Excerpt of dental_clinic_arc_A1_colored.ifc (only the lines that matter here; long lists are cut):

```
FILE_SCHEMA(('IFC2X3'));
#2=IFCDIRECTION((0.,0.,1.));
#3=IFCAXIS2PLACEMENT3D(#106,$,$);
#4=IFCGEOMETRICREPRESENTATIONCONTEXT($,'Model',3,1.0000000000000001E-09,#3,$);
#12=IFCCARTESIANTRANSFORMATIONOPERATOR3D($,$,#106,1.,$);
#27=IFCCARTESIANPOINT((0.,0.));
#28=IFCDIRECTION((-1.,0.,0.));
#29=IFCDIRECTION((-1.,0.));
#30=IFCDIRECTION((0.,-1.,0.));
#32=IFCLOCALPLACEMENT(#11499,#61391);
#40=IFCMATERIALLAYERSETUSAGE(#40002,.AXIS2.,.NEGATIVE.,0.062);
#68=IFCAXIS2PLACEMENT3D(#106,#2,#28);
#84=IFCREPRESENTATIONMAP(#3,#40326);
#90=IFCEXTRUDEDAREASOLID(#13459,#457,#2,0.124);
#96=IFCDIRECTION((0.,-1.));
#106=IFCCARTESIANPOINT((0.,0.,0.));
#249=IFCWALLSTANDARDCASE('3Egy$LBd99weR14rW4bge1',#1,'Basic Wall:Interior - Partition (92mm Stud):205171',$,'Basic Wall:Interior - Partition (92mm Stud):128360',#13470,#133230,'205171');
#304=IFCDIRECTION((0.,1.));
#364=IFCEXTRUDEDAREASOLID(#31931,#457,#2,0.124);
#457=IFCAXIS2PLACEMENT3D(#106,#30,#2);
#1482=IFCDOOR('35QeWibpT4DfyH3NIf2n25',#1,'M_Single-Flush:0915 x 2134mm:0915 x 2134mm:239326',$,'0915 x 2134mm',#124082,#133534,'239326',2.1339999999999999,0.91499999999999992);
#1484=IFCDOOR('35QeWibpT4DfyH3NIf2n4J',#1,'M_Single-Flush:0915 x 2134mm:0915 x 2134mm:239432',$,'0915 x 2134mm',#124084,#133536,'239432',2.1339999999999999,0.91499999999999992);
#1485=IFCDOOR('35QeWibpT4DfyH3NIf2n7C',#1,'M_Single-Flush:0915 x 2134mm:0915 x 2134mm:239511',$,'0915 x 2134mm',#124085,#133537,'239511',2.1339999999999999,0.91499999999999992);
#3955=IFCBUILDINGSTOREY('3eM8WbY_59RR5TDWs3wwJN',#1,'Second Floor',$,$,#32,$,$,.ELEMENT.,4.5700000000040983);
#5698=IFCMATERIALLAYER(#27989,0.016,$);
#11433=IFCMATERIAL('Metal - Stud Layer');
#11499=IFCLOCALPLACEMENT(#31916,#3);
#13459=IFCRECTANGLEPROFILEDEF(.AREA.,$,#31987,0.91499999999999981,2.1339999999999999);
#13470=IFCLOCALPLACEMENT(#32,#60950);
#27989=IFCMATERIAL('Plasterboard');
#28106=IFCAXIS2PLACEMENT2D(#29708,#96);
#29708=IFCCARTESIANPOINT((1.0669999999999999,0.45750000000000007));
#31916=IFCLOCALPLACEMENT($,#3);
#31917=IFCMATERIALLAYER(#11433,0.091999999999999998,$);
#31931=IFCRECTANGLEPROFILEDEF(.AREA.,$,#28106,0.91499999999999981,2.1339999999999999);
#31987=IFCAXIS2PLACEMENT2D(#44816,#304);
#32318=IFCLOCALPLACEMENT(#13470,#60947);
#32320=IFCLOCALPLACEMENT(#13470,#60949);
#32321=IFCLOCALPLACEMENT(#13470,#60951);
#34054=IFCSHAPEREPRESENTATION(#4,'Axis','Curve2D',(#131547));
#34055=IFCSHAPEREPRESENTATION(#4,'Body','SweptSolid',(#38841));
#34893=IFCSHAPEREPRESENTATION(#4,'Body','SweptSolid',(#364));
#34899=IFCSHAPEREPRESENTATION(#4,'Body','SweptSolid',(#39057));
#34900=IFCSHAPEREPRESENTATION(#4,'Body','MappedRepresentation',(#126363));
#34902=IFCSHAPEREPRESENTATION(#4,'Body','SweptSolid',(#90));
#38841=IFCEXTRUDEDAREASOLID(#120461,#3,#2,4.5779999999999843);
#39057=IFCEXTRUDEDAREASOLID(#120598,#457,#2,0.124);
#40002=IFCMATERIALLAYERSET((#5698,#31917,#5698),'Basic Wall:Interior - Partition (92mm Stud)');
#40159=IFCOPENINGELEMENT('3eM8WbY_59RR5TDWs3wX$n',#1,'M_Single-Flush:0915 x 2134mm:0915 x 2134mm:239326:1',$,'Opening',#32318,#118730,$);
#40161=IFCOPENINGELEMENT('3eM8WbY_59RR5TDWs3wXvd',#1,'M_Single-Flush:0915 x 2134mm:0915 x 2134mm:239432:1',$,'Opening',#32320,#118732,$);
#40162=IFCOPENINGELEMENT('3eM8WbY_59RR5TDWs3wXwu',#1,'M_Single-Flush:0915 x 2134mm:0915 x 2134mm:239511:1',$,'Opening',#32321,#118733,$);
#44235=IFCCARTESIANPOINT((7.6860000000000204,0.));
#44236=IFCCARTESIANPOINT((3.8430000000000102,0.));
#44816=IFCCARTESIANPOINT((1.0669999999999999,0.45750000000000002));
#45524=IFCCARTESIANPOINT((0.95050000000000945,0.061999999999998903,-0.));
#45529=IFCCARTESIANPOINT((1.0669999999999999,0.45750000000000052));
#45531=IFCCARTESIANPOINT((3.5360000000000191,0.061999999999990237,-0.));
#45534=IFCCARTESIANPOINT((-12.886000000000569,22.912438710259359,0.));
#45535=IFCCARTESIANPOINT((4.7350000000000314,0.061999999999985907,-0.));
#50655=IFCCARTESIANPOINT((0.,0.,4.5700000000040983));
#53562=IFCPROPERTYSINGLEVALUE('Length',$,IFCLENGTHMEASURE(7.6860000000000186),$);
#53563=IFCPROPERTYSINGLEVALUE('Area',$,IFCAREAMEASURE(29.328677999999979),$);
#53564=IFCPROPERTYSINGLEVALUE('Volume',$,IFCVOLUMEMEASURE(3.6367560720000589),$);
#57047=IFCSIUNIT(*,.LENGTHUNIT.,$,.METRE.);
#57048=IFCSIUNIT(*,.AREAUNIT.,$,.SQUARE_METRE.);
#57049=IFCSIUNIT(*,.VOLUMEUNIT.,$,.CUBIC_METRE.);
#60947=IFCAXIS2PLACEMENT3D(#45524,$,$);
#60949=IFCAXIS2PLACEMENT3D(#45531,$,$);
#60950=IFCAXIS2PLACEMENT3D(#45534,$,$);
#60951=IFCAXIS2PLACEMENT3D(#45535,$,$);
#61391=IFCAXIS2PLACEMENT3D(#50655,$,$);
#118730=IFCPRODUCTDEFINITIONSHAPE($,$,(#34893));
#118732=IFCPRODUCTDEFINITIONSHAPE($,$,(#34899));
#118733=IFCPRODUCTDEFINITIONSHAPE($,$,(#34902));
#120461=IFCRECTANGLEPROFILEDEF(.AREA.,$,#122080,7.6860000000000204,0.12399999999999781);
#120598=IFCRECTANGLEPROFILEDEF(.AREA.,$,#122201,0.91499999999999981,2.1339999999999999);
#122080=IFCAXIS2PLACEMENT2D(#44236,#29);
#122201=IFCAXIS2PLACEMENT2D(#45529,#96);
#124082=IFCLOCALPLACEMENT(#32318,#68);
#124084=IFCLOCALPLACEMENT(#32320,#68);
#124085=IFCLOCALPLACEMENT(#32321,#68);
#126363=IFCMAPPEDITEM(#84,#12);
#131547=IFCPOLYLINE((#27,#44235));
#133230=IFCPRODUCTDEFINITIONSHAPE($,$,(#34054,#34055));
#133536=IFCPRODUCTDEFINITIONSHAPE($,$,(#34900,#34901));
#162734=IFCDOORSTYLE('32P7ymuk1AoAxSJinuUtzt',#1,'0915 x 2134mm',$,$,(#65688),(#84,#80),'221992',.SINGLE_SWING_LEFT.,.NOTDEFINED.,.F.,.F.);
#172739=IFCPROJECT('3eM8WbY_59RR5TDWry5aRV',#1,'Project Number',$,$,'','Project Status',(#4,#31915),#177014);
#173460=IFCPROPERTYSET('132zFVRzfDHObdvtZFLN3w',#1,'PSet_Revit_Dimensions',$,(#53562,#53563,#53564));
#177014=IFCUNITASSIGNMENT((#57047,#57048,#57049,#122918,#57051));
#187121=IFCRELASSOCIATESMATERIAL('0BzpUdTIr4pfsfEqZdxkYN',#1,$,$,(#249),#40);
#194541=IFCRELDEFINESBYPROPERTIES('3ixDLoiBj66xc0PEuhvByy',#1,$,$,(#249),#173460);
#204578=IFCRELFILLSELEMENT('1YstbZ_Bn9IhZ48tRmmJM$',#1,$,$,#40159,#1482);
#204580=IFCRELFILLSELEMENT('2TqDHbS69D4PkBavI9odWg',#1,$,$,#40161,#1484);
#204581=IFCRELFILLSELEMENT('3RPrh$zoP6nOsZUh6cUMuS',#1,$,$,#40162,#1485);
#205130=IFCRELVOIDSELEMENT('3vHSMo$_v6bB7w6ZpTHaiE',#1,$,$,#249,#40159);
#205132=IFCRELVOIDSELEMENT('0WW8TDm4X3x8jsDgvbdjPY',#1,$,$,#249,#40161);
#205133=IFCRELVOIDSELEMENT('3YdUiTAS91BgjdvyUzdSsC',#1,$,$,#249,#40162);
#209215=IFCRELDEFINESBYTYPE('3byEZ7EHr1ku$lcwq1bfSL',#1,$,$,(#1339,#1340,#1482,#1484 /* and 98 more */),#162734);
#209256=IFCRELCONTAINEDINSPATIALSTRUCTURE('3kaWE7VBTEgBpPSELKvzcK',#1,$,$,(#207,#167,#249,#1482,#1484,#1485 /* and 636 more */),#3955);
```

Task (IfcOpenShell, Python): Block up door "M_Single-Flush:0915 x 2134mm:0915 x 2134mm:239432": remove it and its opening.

```python
import ifcopenshell
import ifcopenshell.api.feature
import ifcopenshell.api.pset
import ifcopenshell.api.root
import ifcopenshell.geom
import ifcopenshell.util.element
import ifcopenshell.util.shape
import ifcopenshell.util.unit

model = ifcopenshell.open("dental_clinic_arc_A1_colored.ifc")
area_scale = ifcopenshell.util.unit.calculate_unit_scale(model, "AREAUNIT")
volume_scale = ifcopenshell.util.unit.calculate_unit_scale(model, "VOLUMEUNIT")
settings = ifcopenshell.geom.settings()


def volume(element):
    """Net volume in cubic metres, openings subtracted."""
    shape = ifcopenshell.geom.create_shape(settings, element)
    return ifcopenshell.util.shape.get_volume(shape.geometry)


door = model.by_guid("35QeWibpT4DfyH3NIf2n4J")
opening = door.FillsVoids[0].RelatingOpeningElement
wall = opening.VoidsElements[0].RelatingBuildingElement
before = volume(wall)

ifcopenshell.api.root.remove_product(model, product=door)
ifcopenshell.api.feature.remove_feature(model, feature=opening)

after = volume(wall)
thickness = 0.124  # wall thickness in metres

# Update the wall's stored quantities.
pset = model.by_id(ifcopenshell.util.element.get_pset(wall, "PSet_Revit_Dimensions", should_inherit=False)["id"])
ifcopenshell.api.pset.edit_pset(model, pset=pset, properties={
    "Area": model.create_entity("IfcAreaMeasure", after / thickness / area_scale),
    "Volume": model.create_entity("IfcVolumeMeasure", after / volume_scale),
})

print(f"wall volume {before:.3f} -> {after:.3f} m3")

model.write("dental_clinic_arc_A1_colored-out.ifc")
```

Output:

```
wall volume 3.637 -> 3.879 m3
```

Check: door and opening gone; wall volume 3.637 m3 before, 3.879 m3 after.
